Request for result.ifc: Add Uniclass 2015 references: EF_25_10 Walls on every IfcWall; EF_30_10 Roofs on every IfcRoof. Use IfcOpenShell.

First a look at what the model holds.

```python
import ifcopenshell

model = ifcopenshell.open("result.ifc")
print(model.schema)
print("classifications:", [c.Name for c in model.by_type("IfcClassification")])
for ifc_class in ("IfcDoor", "IfcRoof", "IfcStair", "IfcWall", "IfcWindow"):
    print(ifc_class, len(model.by_type(ifc_class)))
```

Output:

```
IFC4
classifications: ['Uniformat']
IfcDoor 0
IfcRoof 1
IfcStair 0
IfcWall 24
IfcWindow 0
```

```python
import ifcopenshell
import ifcopenshell.api.classification

model = ifcopenshell.open("result.ifc")

system = ifcopenshell.api.classification.add_classification(model, classification="Uniclass 2015")

codes = {
    "IfcWall": ("EF_25_10", "Walls"),
    "IfcRoof": ("EF_30_10", "Roofs"),
}
for ifc_class, (code, name) in codes.items():
    products = model.by_type(ifc_class)
    ifcopenshell.api.classification.add_reference(
        model, products=products, classification=system, identification=code, name=name
    )
    print(code, len(products))

model.write("result_updated.ifc")
```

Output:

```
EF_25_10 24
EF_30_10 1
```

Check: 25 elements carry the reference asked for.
